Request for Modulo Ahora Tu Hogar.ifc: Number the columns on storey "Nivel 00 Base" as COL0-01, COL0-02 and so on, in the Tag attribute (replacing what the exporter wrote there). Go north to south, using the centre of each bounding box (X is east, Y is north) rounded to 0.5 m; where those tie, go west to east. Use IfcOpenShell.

First a look at what the model holds.

```python
import ifcopenshell
import ifcopenshell.util.element
import ifcopenshell.util.placement

model = ifcopenshell.open("Modulo Ahora Tu Hogar.ifc")
print(model.schema)
storey = next(s for s in model.by_type("IfcBuildingStorey") if s.Name == "Nivel 00 Base")
columns = [e for e in ifcopenshell.util.element.get_decomposition(storey) if e.is_a("IfcColumn")]
for e in sorted(columns, key=lambda e: e.id()):
    origin = ifcopenshell.util.placement.get_local_placement(e.ObjectPlacement)[:3, 3]
    print(e.id(), e.Tag, e.Name, origin.round(2) + 0.0, sep=" | ")
```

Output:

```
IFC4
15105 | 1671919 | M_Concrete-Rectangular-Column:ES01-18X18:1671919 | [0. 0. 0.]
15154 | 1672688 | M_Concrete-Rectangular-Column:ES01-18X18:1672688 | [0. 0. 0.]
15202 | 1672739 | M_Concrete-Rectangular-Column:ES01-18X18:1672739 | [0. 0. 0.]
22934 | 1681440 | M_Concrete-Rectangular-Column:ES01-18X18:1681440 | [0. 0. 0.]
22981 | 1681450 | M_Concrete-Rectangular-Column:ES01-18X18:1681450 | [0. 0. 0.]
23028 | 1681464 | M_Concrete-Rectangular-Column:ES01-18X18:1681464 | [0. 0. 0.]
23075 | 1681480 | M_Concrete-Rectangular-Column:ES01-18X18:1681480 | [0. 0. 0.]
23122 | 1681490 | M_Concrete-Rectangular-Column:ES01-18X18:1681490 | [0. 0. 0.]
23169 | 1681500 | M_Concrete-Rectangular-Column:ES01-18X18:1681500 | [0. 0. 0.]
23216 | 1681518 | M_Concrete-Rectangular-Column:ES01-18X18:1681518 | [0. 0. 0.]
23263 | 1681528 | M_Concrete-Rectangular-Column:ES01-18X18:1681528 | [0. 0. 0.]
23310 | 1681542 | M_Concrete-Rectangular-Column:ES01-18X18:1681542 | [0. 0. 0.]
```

```python
import ifcopenshell
import ifcopenshell.geom
import ifcopenshell.util.element
import ifcopenshell.util.shape

model = ifcopenshell.open("Modulo Ahora Tu Hogar.ifc")
settings = ifcopenshell.geom.settings()
settings.set("use-world-coords", True)


def centre(element):
    shape = ifcopenshell.geom.create_shape(settings, element)
    return ifcopenshell.util.shape.get_bbox_centroid(shape.geometry)


storey = next(s for s in model.by_type("IfcBuildingStorey") if s.Name == "Nivel 00 Base")
columns = [e for e in ifcopenshell.util.element.get_decomposition(storey) if e.is_a("IfcColumn")]

# Insertion points can sit at a corner or the storey origin, so sort by the geometry (in metres).
centres = {e: centre(e) for e in columns}
columns.sort(key=lambda e: (-round(centres[e][1] / 0.5), centres[e][0]))

for i, e in enumerate(columns, start=1):
    number = f"COL0-{i:02d}"
    e.Tag = number
    print(e.id(), number)

model.write("Modulo Ahora Tu Hogar-out.ifc")
```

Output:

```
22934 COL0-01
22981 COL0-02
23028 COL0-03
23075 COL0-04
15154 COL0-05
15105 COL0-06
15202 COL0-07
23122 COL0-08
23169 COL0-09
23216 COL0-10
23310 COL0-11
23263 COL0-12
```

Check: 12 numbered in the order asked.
